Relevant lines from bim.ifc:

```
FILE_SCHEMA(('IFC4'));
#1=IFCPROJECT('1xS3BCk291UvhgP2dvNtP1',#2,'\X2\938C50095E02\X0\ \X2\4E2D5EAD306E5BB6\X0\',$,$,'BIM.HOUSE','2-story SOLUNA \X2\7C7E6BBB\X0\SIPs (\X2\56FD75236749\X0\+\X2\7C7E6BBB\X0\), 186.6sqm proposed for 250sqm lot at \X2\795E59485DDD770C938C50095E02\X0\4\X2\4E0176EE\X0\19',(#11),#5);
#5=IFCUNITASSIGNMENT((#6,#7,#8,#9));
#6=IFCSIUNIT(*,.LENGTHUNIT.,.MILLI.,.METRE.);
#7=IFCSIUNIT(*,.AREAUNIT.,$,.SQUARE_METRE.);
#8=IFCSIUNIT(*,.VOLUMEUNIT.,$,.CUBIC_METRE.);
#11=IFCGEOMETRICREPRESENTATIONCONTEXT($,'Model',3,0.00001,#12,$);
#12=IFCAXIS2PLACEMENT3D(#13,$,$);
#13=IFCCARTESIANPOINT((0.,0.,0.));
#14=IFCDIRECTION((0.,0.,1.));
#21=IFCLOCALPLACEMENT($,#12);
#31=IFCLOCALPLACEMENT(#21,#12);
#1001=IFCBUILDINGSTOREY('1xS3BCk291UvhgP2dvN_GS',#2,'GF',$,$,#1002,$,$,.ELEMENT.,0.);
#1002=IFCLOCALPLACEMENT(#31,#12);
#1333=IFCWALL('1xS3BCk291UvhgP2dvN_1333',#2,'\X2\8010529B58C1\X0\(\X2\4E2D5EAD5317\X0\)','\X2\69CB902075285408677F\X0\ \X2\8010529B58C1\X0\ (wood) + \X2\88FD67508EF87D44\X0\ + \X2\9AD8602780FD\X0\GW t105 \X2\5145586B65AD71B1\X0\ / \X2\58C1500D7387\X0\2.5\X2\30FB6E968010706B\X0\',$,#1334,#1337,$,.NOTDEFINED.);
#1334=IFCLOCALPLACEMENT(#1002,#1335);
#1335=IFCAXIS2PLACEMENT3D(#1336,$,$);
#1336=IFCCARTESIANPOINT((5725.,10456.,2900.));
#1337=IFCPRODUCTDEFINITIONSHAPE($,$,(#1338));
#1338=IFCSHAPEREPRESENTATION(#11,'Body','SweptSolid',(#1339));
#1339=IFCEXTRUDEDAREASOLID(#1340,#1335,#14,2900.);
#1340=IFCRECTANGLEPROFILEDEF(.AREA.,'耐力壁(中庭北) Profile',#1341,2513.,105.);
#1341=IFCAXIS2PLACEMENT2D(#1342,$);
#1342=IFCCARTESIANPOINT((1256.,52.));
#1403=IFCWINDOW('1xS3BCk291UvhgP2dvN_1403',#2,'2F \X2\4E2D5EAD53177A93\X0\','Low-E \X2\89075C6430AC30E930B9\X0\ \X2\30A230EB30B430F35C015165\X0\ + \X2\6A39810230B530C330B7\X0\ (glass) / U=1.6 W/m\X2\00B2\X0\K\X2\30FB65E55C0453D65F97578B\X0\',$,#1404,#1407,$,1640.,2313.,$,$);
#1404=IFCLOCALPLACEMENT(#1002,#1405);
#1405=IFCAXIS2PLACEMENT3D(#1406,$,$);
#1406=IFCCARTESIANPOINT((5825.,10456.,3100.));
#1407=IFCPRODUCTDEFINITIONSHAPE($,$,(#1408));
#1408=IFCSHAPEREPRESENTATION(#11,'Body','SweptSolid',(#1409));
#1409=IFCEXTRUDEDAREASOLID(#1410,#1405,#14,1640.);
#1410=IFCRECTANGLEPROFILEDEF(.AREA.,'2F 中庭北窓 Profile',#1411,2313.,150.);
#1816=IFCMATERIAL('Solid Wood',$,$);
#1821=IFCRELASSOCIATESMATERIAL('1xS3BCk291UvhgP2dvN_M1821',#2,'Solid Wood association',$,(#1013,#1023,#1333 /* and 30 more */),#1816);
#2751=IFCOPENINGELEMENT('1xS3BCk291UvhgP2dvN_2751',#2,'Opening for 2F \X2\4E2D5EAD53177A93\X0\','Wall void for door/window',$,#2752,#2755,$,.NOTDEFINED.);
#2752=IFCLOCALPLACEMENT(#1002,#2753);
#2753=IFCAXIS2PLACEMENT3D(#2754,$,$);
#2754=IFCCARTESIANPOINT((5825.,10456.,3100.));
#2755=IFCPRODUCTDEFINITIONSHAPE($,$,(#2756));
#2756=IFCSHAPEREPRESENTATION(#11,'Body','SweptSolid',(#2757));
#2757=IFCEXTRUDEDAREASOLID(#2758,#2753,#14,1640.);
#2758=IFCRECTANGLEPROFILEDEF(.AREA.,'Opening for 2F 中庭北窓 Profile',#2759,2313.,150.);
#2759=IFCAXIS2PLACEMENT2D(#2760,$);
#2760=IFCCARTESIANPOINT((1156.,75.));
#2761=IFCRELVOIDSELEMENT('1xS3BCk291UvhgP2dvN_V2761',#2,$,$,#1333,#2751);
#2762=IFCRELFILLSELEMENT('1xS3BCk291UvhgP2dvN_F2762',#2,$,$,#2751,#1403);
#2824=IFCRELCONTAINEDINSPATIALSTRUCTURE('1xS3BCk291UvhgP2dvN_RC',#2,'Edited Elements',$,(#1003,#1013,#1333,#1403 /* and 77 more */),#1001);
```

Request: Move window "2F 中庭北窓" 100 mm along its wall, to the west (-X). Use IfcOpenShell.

```python
import ifcopenshell
import ifcopenshell.api.geometry
import ifcopenshell.util.placement

model = ifcopenshell.open("bim.ifc")

window = model.by_id(1403)
opening = window.FillsVoids[0].RelatingOpeningElement
wall = opening.VoidsElements[0].RelatingBuildingElement

wall_matrix = ifcopenshell.util.placement.get_local_placement(wall.ObjectPlacement)
shift = wall_matrix[:3, 0] * -100.0
before = ifcopenshell.util.placement.get_local_placement(window.ObjectPlacement)[:3, 3].copy()

# The window is not placed relative to its opening, so move both.
for product in (opening, window):
    matrix = ifcopenshell.util.placement.get_local_placement(product.ObjectPlacement)
    matrix[:3, 3] += shift
    ifcopenshell.api.geometry.edit_object_placement(model, product=product, matrix=matrix, is_si=False)

after = ifcopenshell.util.placement.get_local_placement(window.ObjectPlacement)[:3, 3]
print("window moved by", (after - before).round(3) + 0.0)

model.write("bim-out.ifc")
```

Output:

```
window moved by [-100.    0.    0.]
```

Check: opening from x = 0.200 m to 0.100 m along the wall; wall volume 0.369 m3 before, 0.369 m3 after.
